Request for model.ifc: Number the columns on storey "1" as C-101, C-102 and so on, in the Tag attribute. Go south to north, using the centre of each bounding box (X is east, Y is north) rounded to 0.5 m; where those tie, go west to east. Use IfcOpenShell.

First a look at what the model holds.

```python
import ifcopenshell
import ifcopenshell.util.element
import ifcopenshell.util.placement

model = ifcopenshell.open("model.ifc")
print(model.schema)
storey = next(s for s in model.by_type("IfcBuildingStorey") if s.Name == "1")
columns = [e for e in ifcopenshell.util.element.get_decomposition(storey) if e.is_a("IfcColumn")]
for e in sorted(columns, key=lambda e: e.id()):
    origin = ifcopenshell.util.placement.get_local_placement(e.ObjectPlacement)[:3, 3]
    print(e.id(), e.Tag, e.Name, origin.round(2) + 0.0, sep=" | ")
```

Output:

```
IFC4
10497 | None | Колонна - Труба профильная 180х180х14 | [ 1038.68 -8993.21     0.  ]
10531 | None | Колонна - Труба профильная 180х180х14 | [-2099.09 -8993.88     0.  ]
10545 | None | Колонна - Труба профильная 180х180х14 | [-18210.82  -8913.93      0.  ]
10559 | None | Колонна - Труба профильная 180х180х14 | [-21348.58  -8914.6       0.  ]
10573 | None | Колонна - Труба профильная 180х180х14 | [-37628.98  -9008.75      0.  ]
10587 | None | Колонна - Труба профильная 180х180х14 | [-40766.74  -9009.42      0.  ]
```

```python
import ifcopenshell
import ifcopenshell.geom
import ifcopenshell.util.element
import ifcopenshell.util.shape

model = ifcopenshell.open("model.ifc")
settings = ifcopenshell.geom.settings()
settings.set("use-world-coords", True)


def centre(element):
    shape = ifcopenshell.geom.create_shape(settings, element)
    return ifcopenshell.util.shape.get_bbox_centroid(shape.geometry)


storey = next(s for s in model.by_type("IfcBuildingStorey") if s.Name == "1")
columns = [e for e in ifcopenshell.util.element.get_decomposition(storey) if e.is_a("IfcColumn")]

# Insertion points can sit at a corner or the storey origin, so sort by the geometry (in metres).
centres = {e: centre(e) for e in columns}
columns.sort(key=lambda e: (round(centres[e][1] / 0.5), centres[e][0]))

for i, e in enumerate(columns, start=1):
    number = f"C-1{i:02d}"
    e.Tag = number
    print(e.id(), number)

model.write("model_edited.ifc")
```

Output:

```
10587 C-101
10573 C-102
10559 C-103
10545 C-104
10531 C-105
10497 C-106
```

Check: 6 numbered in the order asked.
